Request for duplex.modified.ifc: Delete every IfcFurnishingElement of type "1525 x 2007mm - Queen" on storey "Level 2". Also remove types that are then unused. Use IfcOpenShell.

First a look at what the model holds.

```python
import ifcopenshell
import ifcopenshell.util.element

model = ifcopenshell.open("duplex.modified.ifc")
print(model.schema)
storey = next(s for s in model.by_type("IfcBuildingStorey") if s.Name == "Level 2")
furniture = [e for e in ifcopenshell.util.element.get_decomposition(storey) if e.is_a("IfcFurnishingElement")]
seen = {}
for e in furniture:
    element_type = ifcopenshell.util.element.get_type(e)
    name = element_type.Name if element_type not in (None, e) else None
    seen[name] = seen.get(name, 0) + 1
for name, count in sorted(seen.items(), key=str):
    print(count, "x", name)
```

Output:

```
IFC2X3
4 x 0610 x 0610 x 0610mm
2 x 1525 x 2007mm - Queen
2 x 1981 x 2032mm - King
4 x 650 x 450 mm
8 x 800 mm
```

```python
import ifcopenshell
import ifcopenshell.api.root
import ifcopenshell.util.element

model = ifcopenshell.open("duplex.modified.ifc")

storey = next(s for s in model.by_type("IfcBuildingStorey") if s.Name == "Level 2")
furniture = [e for e in ifcopenshell.util.element.get_decomposition(storey) if e.is_a("IfcFurnishingElement")]
targets = [e for e in furniture if (t := ifcopenshell.util.element.get_type(e)) not in (None, e) and t.Name == "1525 x 2007mm - Queen"]
types = {ifcopenshell.util.element.get_type(e) for e in targets} - {None, *targets}

for e in targets:
    ifcopenshell.api.root.remove_product(model, product=e)
print(len(targets), "removed")

unused = [t for t in types if not ifcopenshell.util.element.get_types(t)]
for t in unused:
    ifcopenshell.api.root.remove_product(model, product=t)
print(len(unused), "unused types removed")

model.write("duplex.modified_v2.ifc")
```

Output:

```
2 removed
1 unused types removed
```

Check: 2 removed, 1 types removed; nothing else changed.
